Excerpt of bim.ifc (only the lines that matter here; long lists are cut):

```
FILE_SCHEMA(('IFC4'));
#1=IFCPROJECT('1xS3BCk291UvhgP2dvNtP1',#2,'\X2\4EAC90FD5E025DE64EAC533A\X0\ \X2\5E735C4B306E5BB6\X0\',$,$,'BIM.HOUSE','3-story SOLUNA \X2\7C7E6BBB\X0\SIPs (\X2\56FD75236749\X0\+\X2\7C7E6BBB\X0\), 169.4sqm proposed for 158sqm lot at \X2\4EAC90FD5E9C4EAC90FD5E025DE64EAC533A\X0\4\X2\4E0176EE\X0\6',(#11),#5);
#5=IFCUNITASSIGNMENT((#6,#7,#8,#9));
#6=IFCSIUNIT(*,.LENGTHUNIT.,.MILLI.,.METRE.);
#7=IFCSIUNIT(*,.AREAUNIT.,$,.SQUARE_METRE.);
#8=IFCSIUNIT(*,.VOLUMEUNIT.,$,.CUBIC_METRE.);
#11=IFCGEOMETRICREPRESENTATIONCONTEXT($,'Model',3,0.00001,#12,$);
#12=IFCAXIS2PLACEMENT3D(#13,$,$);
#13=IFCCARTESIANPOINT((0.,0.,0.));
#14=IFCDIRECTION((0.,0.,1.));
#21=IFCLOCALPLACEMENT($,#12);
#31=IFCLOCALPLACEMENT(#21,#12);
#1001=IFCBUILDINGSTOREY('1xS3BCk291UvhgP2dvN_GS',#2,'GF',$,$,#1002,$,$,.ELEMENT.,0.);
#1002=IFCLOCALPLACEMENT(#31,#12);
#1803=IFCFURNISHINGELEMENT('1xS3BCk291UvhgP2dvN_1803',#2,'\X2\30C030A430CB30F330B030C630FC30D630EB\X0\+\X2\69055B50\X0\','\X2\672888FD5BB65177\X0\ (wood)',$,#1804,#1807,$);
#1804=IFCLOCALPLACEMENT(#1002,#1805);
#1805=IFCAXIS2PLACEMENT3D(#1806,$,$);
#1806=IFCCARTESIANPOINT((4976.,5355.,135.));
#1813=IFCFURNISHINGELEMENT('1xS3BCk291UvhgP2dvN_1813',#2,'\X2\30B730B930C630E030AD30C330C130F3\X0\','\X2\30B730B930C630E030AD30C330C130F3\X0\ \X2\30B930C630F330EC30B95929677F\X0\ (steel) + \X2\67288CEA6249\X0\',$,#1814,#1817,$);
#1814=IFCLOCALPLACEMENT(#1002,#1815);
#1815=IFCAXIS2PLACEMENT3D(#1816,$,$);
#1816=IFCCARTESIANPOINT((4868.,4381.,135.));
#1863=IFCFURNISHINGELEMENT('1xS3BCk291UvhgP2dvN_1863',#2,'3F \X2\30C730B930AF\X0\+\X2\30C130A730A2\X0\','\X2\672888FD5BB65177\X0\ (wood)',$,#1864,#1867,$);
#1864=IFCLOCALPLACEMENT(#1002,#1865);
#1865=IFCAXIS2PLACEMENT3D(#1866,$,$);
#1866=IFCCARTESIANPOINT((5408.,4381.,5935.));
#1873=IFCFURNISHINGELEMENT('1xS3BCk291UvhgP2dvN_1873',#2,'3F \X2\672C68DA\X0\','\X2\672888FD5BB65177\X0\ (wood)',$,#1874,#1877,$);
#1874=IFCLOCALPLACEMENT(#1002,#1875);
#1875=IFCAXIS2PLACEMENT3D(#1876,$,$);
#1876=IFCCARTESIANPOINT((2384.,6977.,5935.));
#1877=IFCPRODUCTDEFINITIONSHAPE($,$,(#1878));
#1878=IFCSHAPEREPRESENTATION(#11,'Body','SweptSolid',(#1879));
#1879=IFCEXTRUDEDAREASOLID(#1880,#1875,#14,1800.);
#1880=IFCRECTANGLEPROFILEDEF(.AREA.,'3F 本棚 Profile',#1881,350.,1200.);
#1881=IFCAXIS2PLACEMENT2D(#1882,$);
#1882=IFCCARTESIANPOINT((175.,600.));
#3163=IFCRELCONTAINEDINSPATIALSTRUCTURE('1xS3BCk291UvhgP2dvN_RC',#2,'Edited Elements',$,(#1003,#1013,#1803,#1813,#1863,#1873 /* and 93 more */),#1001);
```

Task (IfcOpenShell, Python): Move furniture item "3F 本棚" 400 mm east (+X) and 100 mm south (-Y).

```python
import ifcopenshell
import ifcopenshell.api.geometry
import ifcopenshell.util.placement
import ifcopenshell.util.unit

model = ifcopenshell.open("bim.ifc")
unit_scale = ifcopenshell.util.unit.calculate_unit_scale(model)

item = model.by_id(1873)
matrix = ifcopenshell.util.placement.get_local_placement(item.ObjectPlacement)
matrix[0, 3] += 0.4 / unit_scale
matrix[1, 3] -= 0.1 / unit_scale
ifcopenshell.api.geometry.edit_object_placement(model, product=item, matrix=matrix, is_si=False)

print(ifcopenshell.util.placement.get_local_placement(item.ObjectPlacement).round(3) + 0.0)

model.write("bim-out.ifc")
```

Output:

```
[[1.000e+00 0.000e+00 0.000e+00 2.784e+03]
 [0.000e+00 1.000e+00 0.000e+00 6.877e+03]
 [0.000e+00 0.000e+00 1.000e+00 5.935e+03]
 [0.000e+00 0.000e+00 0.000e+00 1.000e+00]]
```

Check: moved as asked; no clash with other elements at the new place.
